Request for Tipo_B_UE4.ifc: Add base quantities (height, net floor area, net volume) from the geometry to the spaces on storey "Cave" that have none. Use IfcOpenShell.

First a look at what the model holds.

```python
import ifcopenshell
import ifcopenshell.util.element
import ifcopenshell.util.unit

model = ifcopenshell.open("Tipo_B_UE4.ifc")
print(model.schema)
for unit_type in ("LENGTHUNIT", "AREAUNIT", "VOLUMEUNIT"):
    print(unit_type, ifcopenshell.util.unit.calculate_unit_scale(model, unit_type))
storey = next(s for s in model.by_type("IfcBuildingStorey") if s.Name == "Cave")
spaces = [e for e in ifcopenshell.util.element.get_decomposition(storey) if e.is_a("IfcSpace")]
for e in sorted(spaces, key=lambda e: e.id()):
    print(e.id(), e.is_a(), e.Name, list(ifcopenshell.util.element.get_psets(e, qtos_only=True)), sep=" | ")
```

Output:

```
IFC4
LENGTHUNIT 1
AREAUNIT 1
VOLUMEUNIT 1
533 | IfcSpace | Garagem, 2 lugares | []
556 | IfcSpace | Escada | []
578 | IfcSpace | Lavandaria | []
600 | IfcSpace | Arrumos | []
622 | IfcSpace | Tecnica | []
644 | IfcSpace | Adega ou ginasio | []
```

```python
import ifcopenshell
import ifcopenshell.api.pset
import ifcopenshell.geom
import ifcopenshell.util.element
import ifcopenshell.util.shape
import ifcopenshell.util.unit

model = ifcopenshell.open("Tipo_B_UE4.ifc")
unit_scale = ifcopenshell.util.unit.calculate_unit_scale(model)
area_scale = ifcopenshell.util.unit.calculate_unit_scale(model, "AREAUNIT")
volume_scale = ifcopenshell.util.unit.calculate_unit_scale(model, "VOLUMEUNIT")
settings = ifcopenshell.geom.settings()

storey = next(s for s in model.by_type("IfcBuildingStorey") if s.Name == "Cave")
spaces = [e for e in ifcopenshell.util.element.get_decomposition(storey) if e.is_a("IfcSpace")]

for e in sorted(spaces, key=lambda e: e.id()):
    if ifcopenshell.util.element.get_psets(e, qtos_only=True, should_inherit=False):
        continue
    # Geometry comes back in metres, in the element's own axes.
    shape = ifcopenshell.geom.create_shape(settings, e)
    values = {
        "Height": ifcopenshell.util.shape.get_z(shape.geometry) / unit_scale,
        "NetFloorArea": ifcopenshell.util.shape.get_footprint_area(shape.geometry) / area_scale,
        "NetVolume": ifcopenshell.util.shape.get_volume(shape.geometry) / volume_scale,
    }
    qto = ifcopenshell.api.pset.add_qto(model, product=e, name="Qto_SpaceBaseQuantities")
    ifcopenshell.api.pset.edit_qto(model, qto=qto, properties=values)
    print(e.id(), {k: round(v, 3) for k, v in values.items()})

model.write("Tipo_B_UE4-out.ifc")
```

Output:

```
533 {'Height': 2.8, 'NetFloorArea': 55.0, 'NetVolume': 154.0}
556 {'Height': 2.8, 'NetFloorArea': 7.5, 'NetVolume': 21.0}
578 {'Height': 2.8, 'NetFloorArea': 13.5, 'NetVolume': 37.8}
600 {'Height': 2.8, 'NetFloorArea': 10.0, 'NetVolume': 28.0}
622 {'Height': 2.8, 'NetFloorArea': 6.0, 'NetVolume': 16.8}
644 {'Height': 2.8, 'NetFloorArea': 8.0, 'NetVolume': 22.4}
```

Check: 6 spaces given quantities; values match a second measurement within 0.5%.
